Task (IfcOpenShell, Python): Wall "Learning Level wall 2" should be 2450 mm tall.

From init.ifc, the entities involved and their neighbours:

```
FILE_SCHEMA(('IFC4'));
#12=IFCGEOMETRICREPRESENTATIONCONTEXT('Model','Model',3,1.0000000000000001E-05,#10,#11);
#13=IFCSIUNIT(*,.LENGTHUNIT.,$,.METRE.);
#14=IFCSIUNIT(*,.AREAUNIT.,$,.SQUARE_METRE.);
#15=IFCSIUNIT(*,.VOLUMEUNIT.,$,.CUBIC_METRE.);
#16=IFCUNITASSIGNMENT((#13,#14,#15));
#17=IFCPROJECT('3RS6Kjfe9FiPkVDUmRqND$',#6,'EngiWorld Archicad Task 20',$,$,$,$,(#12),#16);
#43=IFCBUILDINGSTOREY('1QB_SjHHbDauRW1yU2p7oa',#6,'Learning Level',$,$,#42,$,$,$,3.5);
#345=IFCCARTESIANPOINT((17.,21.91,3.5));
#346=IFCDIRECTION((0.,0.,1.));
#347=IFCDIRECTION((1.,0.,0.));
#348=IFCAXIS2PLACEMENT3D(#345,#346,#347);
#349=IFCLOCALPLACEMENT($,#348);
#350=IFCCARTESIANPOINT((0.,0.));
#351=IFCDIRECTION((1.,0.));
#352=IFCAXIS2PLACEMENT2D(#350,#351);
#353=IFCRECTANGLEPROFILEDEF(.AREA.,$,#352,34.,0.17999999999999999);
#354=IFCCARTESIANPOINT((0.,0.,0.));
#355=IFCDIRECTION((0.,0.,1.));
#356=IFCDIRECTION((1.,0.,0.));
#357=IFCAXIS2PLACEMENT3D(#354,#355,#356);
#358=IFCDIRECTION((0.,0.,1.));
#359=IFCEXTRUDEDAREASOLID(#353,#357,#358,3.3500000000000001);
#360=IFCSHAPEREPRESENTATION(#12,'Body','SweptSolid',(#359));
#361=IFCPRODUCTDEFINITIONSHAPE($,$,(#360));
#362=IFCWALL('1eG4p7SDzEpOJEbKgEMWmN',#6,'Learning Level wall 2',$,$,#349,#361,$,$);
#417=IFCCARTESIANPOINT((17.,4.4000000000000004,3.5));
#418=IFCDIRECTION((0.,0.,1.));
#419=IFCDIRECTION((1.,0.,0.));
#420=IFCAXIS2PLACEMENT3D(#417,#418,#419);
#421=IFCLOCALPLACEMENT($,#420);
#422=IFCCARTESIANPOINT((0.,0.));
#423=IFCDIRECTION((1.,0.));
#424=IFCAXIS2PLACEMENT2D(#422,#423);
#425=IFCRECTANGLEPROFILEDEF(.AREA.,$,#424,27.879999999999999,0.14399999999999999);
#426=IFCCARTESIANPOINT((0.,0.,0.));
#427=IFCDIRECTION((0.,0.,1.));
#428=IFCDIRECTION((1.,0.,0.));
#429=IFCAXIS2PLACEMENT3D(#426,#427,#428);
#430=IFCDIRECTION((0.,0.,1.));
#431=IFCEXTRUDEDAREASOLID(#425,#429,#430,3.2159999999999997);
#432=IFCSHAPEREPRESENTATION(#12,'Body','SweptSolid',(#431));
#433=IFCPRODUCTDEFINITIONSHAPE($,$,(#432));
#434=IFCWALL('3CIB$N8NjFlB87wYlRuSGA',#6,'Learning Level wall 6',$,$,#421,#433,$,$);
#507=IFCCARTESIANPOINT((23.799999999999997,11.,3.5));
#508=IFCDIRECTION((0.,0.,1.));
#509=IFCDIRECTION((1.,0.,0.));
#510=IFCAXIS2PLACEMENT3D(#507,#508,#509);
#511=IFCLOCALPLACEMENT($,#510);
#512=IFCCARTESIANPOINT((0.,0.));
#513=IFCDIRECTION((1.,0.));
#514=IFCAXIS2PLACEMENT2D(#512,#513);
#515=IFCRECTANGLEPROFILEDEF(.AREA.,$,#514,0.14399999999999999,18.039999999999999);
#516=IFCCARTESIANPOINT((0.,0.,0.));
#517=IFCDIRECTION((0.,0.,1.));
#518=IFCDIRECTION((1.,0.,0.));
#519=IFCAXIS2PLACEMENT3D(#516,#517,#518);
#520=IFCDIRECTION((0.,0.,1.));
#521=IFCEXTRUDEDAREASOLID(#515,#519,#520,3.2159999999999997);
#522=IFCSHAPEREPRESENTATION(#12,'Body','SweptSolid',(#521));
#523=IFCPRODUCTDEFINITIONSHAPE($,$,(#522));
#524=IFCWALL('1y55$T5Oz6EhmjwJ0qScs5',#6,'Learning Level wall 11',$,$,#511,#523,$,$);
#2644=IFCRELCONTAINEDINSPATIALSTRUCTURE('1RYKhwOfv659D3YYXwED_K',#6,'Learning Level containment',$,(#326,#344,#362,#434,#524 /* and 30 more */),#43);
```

```python
import ifcopenshell
import ifcopenshell.geom
import ifcopenshell.util.shape

model = ifcopenshell.open("init.ifc")
settings = ifcopenshell.geom.settings()


def volume(element):
    """Net volume in cubic metres, openings subtracted."""
    shape = ifcopenshell.geom.create_shape(settings, element)
    return ifcopenshell.util.shape.get_volume(shape.geometry)


wall = model.by_id(362)
before = volume(wall)

body = next(r for r in wall.Representation.Representations if r.RepresentationIdentifier == "Body")
solid = body.Items[0]
old_height = solid.Depth
solid.Depth = 2.45
after = volume(wall)

print(f"height {old_height:g} -> {solid.Depth:g}, volume {before:.3f} -> {after:.3f} m3")

model.write("init_v2.ifc")
```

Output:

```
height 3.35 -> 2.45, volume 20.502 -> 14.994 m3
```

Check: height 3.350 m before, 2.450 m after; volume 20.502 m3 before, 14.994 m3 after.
